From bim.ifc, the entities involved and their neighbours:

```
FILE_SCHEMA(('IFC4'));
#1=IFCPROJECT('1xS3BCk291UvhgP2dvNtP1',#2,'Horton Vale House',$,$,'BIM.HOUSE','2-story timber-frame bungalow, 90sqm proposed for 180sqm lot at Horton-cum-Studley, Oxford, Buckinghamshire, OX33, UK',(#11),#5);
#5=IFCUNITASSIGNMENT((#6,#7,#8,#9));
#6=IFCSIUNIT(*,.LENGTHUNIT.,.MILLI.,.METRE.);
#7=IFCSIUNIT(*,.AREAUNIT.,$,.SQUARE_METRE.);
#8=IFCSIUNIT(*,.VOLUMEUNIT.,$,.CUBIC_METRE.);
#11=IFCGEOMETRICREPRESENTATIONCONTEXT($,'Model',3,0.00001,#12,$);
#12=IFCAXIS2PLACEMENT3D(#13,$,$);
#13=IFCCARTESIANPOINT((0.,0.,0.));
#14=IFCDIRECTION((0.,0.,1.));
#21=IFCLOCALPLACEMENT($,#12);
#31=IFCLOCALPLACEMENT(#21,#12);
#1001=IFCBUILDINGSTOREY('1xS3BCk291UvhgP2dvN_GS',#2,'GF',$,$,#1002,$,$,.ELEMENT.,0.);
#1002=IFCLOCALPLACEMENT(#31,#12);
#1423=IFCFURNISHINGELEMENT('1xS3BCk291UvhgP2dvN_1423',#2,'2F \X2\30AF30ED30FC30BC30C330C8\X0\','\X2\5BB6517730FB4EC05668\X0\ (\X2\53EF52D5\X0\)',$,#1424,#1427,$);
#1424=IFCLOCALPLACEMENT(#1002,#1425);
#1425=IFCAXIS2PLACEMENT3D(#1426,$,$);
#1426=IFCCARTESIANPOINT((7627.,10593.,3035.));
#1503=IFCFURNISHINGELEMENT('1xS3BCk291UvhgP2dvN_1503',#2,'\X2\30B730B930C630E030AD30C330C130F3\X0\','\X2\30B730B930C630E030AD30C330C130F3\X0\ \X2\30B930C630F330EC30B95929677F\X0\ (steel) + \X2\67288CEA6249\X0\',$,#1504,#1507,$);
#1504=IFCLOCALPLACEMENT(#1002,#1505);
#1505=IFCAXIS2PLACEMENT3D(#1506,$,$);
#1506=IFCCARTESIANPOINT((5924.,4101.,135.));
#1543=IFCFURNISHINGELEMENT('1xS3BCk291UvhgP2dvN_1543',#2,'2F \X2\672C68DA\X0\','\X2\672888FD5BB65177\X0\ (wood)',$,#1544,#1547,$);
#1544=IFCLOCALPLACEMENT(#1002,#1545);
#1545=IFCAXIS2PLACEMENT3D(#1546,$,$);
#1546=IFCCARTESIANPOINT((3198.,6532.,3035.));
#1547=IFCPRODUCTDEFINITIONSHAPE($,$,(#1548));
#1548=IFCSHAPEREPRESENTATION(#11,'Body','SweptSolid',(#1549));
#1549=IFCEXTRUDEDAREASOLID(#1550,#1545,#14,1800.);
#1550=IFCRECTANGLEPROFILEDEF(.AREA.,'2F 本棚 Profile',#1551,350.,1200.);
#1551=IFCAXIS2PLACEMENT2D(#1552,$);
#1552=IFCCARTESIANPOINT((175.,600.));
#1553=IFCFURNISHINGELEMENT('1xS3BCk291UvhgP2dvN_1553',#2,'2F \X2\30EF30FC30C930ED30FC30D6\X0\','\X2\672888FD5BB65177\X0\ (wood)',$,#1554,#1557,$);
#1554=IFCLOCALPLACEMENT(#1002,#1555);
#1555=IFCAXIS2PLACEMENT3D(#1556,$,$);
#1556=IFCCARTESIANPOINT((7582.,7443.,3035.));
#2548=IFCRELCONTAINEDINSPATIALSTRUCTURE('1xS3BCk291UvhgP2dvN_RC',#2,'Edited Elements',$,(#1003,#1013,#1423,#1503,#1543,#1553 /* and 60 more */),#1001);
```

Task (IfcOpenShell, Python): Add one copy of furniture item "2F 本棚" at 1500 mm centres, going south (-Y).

```python
import numpy as np
import ifcopenshell
import ifcopenshell.api.geometry
import ifcopenshell.api.root
import ifcopenshell.util.element
import ifcopenshell.util.placement
import ifcopenshell.util.unit

model = ifcopenshell.open("bim.ifc")
unit_scale = ifcopenshell.util.unit.calculate_unit_scale(model)


def reuse_history(source, copy):
    """copy_class also copies each property set's owner history, people and application; keep the originals."""
    for rel in copy.IsDefinedBy:
        if rel.is_a("IfcRelDefinesByProperties") and (history := rel.RelatingPropertyDefinition.OwnerHistory):
            rel.RelatingPropertyDefinition.OwnerHistory = source.OwnerHistory
            ifcopenshell.util.element.remove_deep2(model, history)


source = model.by_id(1543)
base = ifcopenshell.util.placement.get_local_placement(source.ObjectPlacement)
step = np.array([0.0, -1.0, 0.0]) * 1.5 / unit_scale

for i in range(1, 2):
    copy = ifcopenshell.api.root.copy_class(model, product=source)
    copy.Representation = ifcopenshell.util.element.copy_deep(
        model, source.Representation, exclude=["IfcGeometricRepresentationContext", "IfcRepresentationMap"]
    )
    reuse_history(source, copy)
    matrix = base.copy()
    matrix[:3, 3] += i * step
    print("added at", matrix[:3, 3].round(3) + 0.0)
    ifcopenshell.api.geometry.edit_object_placement(model, product=copy, matrix=matrix, is_si=False)

model.write("bim_v2.ifc")
```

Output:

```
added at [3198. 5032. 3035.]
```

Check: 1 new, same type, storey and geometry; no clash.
